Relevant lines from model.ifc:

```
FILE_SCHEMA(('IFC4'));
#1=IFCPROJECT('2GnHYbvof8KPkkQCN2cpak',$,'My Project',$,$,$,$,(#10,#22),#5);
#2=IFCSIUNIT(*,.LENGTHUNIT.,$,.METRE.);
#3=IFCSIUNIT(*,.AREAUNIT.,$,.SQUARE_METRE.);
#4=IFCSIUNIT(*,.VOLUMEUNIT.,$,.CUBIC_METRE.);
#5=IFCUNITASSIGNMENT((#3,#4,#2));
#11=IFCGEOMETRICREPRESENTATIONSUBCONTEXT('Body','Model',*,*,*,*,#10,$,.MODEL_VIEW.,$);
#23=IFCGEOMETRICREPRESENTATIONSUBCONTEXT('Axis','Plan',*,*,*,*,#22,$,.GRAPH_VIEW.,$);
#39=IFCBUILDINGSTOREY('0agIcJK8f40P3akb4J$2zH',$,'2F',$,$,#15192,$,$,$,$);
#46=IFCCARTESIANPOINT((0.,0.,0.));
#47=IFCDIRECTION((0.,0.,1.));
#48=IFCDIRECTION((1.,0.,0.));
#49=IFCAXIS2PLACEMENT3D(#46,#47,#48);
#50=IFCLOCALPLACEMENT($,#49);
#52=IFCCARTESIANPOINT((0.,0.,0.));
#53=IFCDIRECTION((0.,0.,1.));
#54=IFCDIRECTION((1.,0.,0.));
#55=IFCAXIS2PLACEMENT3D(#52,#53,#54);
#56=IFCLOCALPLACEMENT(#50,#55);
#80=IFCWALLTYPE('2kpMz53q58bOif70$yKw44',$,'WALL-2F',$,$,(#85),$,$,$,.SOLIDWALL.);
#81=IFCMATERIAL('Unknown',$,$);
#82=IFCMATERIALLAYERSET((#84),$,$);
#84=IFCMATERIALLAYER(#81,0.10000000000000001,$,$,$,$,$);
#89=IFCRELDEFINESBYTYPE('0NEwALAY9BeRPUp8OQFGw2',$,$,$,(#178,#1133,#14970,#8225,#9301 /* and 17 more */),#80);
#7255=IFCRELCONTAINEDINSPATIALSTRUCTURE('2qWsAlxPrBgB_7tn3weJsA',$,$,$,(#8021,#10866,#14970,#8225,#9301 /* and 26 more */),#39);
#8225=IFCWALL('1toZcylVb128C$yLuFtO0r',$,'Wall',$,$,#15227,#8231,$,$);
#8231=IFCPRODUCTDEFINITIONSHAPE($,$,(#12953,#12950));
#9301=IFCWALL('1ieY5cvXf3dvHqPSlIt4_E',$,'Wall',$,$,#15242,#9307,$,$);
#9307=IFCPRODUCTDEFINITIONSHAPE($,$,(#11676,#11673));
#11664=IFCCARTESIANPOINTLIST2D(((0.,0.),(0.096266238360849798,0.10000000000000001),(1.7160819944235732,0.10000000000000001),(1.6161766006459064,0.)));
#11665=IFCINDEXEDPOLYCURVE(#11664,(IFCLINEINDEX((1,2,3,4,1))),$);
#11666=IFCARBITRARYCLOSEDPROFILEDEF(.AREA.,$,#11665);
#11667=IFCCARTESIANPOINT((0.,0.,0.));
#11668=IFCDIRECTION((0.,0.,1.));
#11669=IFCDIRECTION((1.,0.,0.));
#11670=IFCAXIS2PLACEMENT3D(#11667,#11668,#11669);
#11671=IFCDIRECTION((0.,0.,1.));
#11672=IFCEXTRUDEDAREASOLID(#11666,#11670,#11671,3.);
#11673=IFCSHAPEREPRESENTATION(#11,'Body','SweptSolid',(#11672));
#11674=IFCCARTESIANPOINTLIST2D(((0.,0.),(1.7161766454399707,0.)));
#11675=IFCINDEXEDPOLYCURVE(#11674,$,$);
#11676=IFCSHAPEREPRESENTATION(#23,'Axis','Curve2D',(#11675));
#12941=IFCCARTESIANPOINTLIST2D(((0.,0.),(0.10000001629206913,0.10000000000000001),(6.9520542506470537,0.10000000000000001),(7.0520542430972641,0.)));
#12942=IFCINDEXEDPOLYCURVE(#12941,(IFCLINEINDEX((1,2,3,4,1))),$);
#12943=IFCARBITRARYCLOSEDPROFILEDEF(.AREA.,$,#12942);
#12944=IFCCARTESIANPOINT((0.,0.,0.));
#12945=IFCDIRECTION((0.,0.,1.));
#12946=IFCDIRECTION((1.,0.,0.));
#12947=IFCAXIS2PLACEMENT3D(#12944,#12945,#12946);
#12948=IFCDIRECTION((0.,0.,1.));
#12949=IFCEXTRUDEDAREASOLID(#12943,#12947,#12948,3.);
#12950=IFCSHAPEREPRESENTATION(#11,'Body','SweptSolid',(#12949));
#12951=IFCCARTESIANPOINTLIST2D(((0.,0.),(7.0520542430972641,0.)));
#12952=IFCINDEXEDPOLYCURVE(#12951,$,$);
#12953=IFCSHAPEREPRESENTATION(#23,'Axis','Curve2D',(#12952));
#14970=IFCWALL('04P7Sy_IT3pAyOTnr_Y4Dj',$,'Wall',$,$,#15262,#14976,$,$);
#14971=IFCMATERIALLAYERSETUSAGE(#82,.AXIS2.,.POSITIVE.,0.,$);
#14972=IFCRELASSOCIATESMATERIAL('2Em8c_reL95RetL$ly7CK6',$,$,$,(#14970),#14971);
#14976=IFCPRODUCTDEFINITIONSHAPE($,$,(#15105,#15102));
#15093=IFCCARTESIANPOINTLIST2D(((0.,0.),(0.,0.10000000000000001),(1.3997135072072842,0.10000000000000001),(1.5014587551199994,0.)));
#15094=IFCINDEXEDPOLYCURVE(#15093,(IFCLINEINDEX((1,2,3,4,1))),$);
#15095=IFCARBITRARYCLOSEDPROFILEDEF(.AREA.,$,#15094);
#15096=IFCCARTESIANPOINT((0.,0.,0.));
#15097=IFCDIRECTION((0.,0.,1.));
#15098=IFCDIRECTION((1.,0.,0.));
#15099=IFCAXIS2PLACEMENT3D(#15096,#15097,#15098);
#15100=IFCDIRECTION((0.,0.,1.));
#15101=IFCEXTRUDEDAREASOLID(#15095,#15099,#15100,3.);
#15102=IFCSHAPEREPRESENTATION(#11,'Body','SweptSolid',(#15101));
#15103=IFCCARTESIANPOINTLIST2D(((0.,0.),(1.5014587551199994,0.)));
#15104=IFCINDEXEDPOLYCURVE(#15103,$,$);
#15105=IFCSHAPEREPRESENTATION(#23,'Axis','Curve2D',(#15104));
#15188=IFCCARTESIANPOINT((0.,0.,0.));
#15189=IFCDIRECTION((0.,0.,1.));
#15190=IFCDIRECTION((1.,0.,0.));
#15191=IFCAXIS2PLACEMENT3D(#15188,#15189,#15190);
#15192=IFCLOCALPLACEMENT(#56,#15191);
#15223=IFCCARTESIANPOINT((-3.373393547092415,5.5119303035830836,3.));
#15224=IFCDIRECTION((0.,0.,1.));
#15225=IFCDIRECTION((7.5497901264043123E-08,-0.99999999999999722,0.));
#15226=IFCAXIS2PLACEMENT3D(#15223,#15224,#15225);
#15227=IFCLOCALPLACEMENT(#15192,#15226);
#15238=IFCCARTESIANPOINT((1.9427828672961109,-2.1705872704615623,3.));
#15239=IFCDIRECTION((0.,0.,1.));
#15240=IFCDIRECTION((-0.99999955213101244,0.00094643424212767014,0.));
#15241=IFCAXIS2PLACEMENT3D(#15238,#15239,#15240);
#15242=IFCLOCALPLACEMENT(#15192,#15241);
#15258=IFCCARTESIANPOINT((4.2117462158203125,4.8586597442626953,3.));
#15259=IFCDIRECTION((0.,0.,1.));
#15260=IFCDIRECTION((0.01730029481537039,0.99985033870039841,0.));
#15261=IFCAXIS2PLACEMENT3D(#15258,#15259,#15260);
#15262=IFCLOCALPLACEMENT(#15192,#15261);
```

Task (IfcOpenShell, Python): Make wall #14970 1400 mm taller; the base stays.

```python
import ifcopenshell
import ifcopenshell.geom
import ifcopenshell.util.representation
import ifcopenshell.util.shape

model = ifcopenshell.open("model.ifc")
settings = ifcopenshell.geom.settings()


def volume(element):
    """Net volume in cubic metres, openings subtracted."""
    shape = ifcopenshell.geom.create_shape(settings, element)
    return ifcopenshell.util.shape.get_volume(shape.geometry)


wall = model.by_guid("04P7Sy_IT3pAyOTnr_Y4Dj")
before = volume(wall)

body = ifcopenshell.util.representation.get_representation(wall, "Model", "Body")
solid = body.Items[0]
old_height = solid.Depth
solid.Depth += 1.4
after = volume(wall)

print(f"height {old_height:g} -> {solid.Depth:g}, volume {before:.3f} -> {after:.3f} m3")

model.write("model_v2.ifc")
```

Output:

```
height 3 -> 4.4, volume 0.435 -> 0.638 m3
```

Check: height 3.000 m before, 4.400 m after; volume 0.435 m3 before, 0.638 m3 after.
